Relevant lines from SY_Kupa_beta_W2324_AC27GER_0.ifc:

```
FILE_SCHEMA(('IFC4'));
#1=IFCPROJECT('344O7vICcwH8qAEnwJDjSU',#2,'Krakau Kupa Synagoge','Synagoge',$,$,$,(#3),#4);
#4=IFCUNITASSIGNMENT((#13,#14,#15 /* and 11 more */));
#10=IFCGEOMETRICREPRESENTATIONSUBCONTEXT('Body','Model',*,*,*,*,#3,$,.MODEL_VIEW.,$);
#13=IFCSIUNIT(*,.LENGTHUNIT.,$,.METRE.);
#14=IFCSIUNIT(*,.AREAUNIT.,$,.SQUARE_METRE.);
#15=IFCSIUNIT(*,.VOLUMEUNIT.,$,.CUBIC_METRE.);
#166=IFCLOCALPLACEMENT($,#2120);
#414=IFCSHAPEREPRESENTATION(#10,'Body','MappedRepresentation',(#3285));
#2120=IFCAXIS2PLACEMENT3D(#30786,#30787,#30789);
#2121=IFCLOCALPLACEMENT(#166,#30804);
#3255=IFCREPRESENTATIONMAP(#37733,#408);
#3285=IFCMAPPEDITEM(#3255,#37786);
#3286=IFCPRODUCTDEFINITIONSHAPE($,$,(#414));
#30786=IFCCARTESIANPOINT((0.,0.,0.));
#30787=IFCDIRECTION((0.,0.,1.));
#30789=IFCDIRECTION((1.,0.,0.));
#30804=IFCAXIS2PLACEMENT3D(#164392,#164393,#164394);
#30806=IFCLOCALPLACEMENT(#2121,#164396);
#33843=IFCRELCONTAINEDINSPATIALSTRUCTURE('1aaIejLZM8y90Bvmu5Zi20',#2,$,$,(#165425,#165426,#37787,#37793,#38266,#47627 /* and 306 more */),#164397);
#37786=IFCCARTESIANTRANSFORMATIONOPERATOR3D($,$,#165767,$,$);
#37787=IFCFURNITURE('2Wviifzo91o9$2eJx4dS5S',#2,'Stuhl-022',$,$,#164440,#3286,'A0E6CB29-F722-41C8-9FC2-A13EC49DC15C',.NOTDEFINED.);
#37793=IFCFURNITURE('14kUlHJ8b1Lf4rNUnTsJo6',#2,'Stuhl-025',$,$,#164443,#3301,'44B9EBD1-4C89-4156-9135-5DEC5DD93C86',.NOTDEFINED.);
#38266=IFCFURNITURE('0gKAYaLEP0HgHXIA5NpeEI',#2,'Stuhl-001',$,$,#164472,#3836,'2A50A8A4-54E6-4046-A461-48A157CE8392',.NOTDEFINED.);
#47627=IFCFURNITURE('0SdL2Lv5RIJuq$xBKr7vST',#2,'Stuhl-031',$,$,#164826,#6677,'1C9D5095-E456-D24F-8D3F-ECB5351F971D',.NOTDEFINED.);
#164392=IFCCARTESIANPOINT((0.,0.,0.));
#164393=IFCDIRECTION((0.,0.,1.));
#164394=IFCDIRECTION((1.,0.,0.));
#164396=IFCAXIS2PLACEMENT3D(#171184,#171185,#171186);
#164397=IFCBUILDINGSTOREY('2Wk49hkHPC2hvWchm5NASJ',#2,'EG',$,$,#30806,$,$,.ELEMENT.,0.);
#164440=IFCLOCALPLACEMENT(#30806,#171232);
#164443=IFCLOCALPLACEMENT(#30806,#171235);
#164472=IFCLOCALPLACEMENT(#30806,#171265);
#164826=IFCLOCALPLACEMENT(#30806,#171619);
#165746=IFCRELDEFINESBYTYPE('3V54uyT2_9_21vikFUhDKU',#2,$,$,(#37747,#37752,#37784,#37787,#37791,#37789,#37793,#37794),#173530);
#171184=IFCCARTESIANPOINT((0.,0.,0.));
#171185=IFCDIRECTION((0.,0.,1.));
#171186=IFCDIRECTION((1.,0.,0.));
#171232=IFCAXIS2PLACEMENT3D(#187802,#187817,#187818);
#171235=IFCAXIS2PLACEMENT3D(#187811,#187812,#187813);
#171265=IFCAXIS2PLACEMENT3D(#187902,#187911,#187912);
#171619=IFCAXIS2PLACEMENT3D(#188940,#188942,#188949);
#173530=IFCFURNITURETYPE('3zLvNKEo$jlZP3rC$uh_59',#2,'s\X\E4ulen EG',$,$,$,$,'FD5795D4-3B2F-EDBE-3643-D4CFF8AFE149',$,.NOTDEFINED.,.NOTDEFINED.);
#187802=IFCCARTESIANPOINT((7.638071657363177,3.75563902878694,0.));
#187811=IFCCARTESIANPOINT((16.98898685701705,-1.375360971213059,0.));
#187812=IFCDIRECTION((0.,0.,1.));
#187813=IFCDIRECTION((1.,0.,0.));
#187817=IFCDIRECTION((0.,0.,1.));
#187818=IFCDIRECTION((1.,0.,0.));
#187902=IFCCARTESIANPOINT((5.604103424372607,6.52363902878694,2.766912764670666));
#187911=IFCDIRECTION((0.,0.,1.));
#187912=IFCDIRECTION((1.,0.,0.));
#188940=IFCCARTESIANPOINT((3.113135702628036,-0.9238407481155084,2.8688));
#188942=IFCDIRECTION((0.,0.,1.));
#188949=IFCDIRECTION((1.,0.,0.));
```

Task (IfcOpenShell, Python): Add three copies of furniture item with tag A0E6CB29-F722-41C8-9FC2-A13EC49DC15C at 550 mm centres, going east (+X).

```python
import numpy as np
import ifcopenshell
import ifcopenshell.api.geometry
import ifcopenshell.api.root
import ifcopenshell.util.element
import ifcopenshell.util.placement
import ifcopenshell.util.unit

model = ifcopenshell.open("SY_Kupa_beta_W2324_AC27GER_0.ifc")
unit_scale = ifcopenshell.util.unit.calculate_unit_scale(model)


def reuse_history(source, copy):
    """copy_class also copies each property set's owner history, people and application; keep the originals."""
    for rel in copy.IsDefinedBy:
        if rel.is_a("IfcRelDefinesByProperties") and (history := rel.RelatingPropertyDefinition.OwnerHistory):
            rel.RelatingPropertyDefinition.OwnerHistory = source.OwnerHistory
            ifcopenshell.util.element.remove_deep2(model, history)


source = model.by_id(37787)
base = ifcopenshell.util.placement.get_local_placement(source.ObjectPlacement)
step = np.array([1.0, 0.0, 0.0]) * 0.55 / unit_scale

for i in range(1, 4):
    copy = ifcopenshell.api.root.copy_class(model, product=source)
    copy.Representation = ifcopenshell.util.element.copy_deep(
        model, source.Representation, exclude=["IfcGeometricRepresentationContext", "IfcRepresentationMap"]
    )
    copy.Tag = None
    reuse_history(source, copy)
    matrix = base.copy()
    matrix[:3, 3] += i * step
    print("added at", matrix[:3, 3].round(3) + 0.0)
    ifcopenshell.api.geometry.edit_object_placement(model, product=copy, matrix=matrix, is_si=False)

model.write("SY_Kupa_beta_W2324_AC27GER_0_updated.ifc")
```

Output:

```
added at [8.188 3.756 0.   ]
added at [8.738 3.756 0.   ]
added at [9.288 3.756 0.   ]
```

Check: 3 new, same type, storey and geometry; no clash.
